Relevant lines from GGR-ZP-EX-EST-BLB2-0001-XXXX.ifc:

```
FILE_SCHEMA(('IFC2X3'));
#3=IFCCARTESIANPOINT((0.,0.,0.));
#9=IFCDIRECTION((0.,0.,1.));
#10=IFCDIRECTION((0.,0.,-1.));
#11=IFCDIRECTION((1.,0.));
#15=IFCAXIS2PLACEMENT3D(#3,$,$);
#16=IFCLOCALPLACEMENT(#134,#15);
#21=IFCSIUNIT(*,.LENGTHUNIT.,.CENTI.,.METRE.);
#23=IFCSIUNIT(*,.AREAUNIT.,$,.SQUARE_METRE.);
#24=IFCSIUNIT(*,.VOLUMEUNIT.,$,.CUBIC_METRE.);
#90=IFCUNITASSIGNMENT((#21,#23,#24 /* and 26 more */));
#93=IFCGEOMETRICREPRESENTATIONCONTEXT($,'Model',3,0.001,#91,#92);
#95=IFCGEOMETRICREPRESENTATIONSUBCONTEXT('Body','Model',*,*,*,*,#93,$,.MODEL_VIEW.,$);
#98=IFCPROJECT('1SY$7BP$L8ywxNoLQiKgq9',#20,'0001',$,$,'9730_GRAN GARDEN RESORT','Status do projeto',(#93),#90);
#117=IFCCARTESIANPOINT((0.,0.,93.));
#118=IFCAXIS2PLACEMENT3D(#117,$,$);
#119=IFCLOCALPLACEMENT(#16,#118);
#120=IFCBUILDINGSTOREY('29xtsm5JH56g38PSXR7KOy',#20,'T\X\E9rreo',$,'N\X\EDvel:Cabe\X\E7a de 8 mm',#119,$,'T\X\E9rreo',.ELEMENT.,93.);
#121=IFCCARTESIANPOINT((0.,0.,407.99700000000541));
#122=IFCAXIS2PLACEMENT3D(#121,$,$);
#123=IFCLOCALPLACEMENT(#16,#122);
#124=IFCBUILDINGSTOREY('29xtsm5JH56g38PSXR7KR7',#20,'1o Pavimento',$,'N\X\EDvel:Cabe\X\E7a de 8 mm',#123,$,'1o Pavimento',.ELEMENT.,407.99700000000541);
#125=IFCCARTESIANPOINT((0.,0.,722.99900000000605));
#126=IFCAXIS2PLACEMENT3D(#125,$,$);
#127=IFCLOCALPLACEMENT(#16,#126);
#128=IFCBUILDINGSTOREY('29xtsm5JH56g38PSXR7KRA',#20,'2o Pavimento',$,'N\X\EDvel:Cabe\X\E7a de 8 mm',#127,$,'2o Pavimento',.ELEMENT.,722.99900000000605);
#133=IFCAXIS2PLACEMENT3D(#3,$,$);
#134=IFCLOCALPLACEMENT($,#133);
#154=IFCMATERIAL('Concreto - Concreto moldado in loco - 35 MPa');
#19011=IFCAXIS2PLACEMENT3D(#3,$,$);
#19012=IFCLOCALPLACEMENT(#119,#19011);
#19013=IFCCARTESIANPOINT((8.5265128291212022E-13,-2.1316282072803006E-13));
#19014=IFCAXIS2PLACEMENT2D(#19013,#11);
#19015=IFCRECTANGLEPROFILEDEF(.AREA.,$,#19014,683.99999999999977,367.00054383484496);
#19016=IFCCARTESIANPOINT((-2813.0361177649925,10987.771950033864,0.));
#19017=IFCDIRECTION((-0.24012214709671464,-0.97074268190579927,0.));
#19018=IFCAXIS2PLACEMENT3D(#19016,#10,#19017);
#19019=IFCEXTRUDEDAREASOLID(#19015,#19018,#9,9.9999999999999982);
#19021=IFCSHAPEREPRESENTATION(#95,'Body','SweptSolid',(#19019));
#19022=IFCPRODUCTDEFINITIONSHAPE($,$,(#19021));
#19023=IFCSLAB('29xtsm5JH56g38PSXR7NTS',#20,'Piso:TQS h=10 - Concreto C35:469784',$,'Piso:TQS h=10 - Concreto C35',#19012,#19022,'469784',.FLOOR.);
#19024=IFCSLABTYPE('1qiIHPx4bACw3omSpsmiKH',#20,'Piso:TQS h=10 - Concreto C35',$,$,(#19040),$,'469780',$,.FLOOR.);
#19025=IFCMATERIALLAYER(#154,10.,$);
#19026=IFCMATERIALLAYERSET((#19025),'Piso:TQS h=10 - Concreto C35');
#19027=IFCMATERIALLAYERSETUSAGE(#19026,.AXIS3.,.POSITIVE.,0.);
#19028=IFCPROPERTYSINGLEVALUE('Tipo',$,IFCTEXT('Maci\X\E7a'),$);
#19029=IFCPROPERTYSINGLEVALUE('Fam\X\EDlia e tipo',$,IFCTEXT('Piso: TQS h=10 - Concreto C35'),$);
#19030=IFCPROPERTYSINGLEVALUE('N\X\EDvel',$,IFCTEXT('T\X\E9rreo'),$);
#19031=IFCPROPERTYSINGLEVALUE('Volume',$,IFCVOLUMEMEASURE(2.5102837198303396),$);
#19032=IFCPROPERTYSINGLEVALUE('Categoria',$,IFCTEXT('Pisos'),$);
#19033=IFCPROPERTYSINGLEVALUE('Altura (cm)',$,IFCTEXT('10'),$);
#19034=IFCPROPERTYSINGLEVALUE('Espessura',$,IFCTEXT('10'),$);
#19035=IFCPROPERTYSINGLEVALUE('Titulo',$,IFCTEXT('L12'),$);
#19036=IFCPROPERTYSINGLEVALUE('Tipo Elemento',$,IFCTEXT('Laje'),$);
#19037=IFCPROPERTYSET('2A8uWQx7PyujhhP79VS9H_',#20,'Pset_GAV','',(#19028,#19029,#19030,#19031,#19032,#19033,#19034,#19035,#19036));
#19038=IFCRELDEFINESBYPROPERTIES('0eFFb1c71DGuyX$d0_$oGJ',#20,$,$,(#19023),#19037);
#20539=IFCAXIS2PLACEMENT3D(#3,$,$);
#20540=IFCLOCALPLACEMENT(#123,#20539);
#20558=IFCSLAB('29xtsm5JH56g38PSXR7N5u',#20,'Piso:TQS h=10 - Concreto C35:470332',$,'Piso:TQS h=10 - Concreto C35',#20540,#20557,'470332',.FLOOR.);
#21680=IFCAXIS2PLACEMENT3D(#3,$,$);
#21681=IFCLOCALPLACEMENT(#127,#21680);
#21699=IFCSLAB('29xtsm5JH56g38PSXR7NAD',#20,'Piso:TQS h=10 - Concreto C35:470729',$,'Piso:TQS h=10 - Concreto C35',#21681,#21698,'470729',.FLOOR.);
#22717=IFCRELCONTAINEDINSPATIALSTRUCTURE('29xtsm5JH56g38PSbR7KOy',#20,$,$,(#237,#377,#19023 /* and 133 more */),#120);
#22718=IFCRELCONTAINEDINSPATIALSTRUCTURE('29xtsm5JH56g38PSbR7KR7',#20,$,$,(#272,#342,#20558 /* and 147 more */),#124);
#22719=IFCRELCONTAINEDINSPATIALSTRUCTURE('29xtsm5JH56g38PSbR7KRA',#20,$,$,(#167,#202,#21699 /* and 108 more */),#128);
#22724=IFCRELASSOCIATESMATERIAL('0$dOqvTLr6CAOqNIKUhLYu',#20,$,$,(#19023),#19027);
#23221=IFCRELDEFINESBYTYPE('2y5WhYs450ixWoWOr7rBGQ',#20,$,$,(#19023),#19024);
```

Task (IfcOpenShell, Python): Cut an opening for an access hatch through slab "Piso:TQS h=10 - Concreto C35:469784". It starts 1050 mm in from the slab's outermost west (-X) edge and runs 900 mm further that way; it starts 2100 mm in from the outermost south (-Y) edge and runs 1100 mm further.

```python
import numpy as np
import ifcopenshell
import ifcopenshell.api.feature
import ifcopenshell.api.geometry
import ifcopenshell.api.pset
import ifcopenshell.api.root
import ifcopenshell.geom
import ifcopenshell.util.element
import ifcopenshell.util.placement
import ifcopenshell.util.representation
import ifcopenshell.util.shape
import ifcopenshell.util.unit

model = ifcopenshell.open("GGR-ZP-EX-EST-BLB2-0001-XXXX.ifc")
unit_scale = ifcopenshell.util.unit.calculate_unit_scale(model)
volume_scale = ifcopenshell.util.unit.calculate_unit_scale(model, "VOLUMEUNIT")
settings = ifcopenshell.geom.settings()


def volume(element):
    """Net volume in cubic metres, openings subtracted."""
    shape = ifcopenshell.geom.create_shape(settings, element)
    return ifcopenshell.util.shape.get_volume(shape.geometry)


slab = model.by_guid("29xtsm5JH56g38PSXR7NTS")
before = volume(slab)

# Extent in the slab's own axes, in metres. The edges named are its -X and -Y sides.
slab_shape = ifcopenshell.geom.create_shape(settings, slab)
vertices = ifcopenshell.util.shape.get_vertices(slab_shape.geometry)
x_min, y_min, bottom = vertices.min(axis=0)
top = vertices[:, 2].max()

opening = ifcopenshell.api.root.create_entity(model, ifc_class="IfcOpeningElement", name="Access hatch opening")
context = ifcopenshell.util.representation.get_context(model, "Model", "Body", "MODEL_VIEW")
width, depth = 0.9, 1.1
outline = [(0.0, 0.0), (width, 0.0), (width, depth), (0.0, depth), (0.0, 0.0)]
# Overshoot both faces by 50 mm so the cut is clean.
shape = ifcopenshell.api.geometry.add_slab_representation(
    model, context=context, depth=top - bottom + 0.1, polyline=outline
)
ifcopenshell.api.geometry.assign_representation(model, product=opening, representation=shape)

matrix = ifcopenshell.util.placement.get_local_placement(slab.ObjectPlacement)
matrix[:, 3] = matrix @ np.append(np.array([x_min + 1.05, y_min + 2.1, bottom - 0.05]) / unit_scale, 1.0)
ifcopenshell.api.geometry.edit_object_placement(model, product=opening, matrix=matrix, is_si=False)
ifcopenshell.api.feature.add_feature(model, feature=opening, element=slab)

after = volume(slab)

# Update the slab's stored quantities.
pset = model.by_id(ifcopenshell.util.element.get_pset(slab, "Pset_GAV", should_inherit=False)["id"])
ifcopenshell.api.pset.edit_pset(model, pset=pset, properties={
    "Volume": model.create_entity("IfcVolumeMeasure", after / volume_scale),
})

print(f"slab volume {before:.3f} -> {after:.3f} m3")

model.write("GGR-ZP-EX-EST-BLB2-0001-XXXX_v2.ifc")
```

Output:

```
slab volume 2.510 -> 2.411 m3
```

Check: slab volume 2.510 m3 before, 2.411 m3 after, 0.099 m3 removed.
